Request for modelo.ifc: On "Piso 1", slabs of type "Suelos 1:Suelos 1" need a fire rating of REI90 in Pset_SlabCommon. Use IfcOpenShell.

First a look at what the model holds.

```python
import ifcopenshell
import ifcopenshell.util.element

model = ifcopenshell.open("modelo.ifc")
print(model.schema)
storey = next(s for s in model.by_type("IfcBuildingStorey") if s.Name == "Piso 1")
slabs = [e for e in ifcopenshell.util.element.get_decomposition(storey) if e.is_a("IfcSlab")]
seen = {}
for e in slabs:
    element_type = ifcopenshell.util.element.get_type(e)
    key = (element_type.Name if element_type != e and element_type else None, ifcopenshell.util.element.get_pset(e, "Pset_SlabCommon", "FireRating"))
    seen[key] = seen.get(key, 0) + 1
for (name, value), count in sorted(seen.items(), key=str):
    print(count, "x", name, "|", value)
```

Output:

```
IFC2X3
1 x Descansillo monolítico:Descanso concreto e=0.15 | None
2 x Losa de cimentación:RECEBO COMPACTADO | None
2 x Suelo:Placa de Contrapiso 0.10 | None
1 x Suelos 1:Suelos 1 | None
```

```python
import ifcopenshell
import ifcopenshell.api.pset
import ifcopenshell.util.element

model = ifcopenshell.open("modelo.ifc")

storey = next(s for s in model.by_type("IfcBuildingStorey") if s.Name == "Piso 1")
slabs = [e for e in ifcopenshell.util.element.get_decomposition(storey) if e.is_a("IfcSlab")]

count = 0
for e in slabs:
    element_type = ifcopenshell.util.element.get_type(e)
    if element_type in (None, e) or element_type.Name != "Suelos 1:Suelos 1":
        continue
    # add_pset returns the element's existing set when there is one.
    pset = ifcopenshell.api.pset.add_pset(model, product=e, name="Pset_SlabCommon")
    ifcopenshell.api.pset.edit_pset(model, pset=pset, properties={"FireRating": "REI90"})
    count += 1

print(count, "slabs updated")

model.write("modelo_updated.ifc")
```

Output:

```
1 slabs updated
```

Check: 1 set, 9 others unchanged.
